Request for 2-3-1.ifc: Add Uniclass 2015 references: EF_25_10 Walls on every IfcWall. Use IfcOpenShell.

First a look at what the model holds.

```python
import ifcopenshell

model = ifcopenshell.open("2-3-1.ifc")
print(model.schema)
print("classifications:", [c.Name for c in model.by_type("IfcClassification")])
for ifc_class in ("IfcDoor", "IfcRoof", "IfcStair", "IfcWall", "IfcWindow"):
    print(ifc_class, len(model.by_type(ifc_class)))
```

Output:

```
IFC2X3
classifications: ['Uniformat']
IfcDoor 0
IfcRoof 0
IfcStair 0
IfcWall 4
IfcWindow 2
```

```python
import ifcopenshell
import ifcopenshell.api.classification

model = ifcopenshell.open("2-3-1.ifc")

# IFC2X3 requires Source and Edition and has no link from the project to the system.
system = model.create_entity("IfcClassification", Source="NBS", Edition="2015", Name="Uniclass 2015")

codes = {
    "IfcWall": ("EF_25_10", "Walls"),
}
for ifc_class, (code, name) in codes.items():
    products = model.by_type(ifc_class)
    ifcopenshell.api.classification.add_reference(
        model, products=products, classification=system, identification=code, name=name
    )
    print(code, len(products))

model.write("2-3-1_v2.ifc")
```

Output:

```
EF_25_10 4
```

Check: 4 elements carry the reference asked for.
